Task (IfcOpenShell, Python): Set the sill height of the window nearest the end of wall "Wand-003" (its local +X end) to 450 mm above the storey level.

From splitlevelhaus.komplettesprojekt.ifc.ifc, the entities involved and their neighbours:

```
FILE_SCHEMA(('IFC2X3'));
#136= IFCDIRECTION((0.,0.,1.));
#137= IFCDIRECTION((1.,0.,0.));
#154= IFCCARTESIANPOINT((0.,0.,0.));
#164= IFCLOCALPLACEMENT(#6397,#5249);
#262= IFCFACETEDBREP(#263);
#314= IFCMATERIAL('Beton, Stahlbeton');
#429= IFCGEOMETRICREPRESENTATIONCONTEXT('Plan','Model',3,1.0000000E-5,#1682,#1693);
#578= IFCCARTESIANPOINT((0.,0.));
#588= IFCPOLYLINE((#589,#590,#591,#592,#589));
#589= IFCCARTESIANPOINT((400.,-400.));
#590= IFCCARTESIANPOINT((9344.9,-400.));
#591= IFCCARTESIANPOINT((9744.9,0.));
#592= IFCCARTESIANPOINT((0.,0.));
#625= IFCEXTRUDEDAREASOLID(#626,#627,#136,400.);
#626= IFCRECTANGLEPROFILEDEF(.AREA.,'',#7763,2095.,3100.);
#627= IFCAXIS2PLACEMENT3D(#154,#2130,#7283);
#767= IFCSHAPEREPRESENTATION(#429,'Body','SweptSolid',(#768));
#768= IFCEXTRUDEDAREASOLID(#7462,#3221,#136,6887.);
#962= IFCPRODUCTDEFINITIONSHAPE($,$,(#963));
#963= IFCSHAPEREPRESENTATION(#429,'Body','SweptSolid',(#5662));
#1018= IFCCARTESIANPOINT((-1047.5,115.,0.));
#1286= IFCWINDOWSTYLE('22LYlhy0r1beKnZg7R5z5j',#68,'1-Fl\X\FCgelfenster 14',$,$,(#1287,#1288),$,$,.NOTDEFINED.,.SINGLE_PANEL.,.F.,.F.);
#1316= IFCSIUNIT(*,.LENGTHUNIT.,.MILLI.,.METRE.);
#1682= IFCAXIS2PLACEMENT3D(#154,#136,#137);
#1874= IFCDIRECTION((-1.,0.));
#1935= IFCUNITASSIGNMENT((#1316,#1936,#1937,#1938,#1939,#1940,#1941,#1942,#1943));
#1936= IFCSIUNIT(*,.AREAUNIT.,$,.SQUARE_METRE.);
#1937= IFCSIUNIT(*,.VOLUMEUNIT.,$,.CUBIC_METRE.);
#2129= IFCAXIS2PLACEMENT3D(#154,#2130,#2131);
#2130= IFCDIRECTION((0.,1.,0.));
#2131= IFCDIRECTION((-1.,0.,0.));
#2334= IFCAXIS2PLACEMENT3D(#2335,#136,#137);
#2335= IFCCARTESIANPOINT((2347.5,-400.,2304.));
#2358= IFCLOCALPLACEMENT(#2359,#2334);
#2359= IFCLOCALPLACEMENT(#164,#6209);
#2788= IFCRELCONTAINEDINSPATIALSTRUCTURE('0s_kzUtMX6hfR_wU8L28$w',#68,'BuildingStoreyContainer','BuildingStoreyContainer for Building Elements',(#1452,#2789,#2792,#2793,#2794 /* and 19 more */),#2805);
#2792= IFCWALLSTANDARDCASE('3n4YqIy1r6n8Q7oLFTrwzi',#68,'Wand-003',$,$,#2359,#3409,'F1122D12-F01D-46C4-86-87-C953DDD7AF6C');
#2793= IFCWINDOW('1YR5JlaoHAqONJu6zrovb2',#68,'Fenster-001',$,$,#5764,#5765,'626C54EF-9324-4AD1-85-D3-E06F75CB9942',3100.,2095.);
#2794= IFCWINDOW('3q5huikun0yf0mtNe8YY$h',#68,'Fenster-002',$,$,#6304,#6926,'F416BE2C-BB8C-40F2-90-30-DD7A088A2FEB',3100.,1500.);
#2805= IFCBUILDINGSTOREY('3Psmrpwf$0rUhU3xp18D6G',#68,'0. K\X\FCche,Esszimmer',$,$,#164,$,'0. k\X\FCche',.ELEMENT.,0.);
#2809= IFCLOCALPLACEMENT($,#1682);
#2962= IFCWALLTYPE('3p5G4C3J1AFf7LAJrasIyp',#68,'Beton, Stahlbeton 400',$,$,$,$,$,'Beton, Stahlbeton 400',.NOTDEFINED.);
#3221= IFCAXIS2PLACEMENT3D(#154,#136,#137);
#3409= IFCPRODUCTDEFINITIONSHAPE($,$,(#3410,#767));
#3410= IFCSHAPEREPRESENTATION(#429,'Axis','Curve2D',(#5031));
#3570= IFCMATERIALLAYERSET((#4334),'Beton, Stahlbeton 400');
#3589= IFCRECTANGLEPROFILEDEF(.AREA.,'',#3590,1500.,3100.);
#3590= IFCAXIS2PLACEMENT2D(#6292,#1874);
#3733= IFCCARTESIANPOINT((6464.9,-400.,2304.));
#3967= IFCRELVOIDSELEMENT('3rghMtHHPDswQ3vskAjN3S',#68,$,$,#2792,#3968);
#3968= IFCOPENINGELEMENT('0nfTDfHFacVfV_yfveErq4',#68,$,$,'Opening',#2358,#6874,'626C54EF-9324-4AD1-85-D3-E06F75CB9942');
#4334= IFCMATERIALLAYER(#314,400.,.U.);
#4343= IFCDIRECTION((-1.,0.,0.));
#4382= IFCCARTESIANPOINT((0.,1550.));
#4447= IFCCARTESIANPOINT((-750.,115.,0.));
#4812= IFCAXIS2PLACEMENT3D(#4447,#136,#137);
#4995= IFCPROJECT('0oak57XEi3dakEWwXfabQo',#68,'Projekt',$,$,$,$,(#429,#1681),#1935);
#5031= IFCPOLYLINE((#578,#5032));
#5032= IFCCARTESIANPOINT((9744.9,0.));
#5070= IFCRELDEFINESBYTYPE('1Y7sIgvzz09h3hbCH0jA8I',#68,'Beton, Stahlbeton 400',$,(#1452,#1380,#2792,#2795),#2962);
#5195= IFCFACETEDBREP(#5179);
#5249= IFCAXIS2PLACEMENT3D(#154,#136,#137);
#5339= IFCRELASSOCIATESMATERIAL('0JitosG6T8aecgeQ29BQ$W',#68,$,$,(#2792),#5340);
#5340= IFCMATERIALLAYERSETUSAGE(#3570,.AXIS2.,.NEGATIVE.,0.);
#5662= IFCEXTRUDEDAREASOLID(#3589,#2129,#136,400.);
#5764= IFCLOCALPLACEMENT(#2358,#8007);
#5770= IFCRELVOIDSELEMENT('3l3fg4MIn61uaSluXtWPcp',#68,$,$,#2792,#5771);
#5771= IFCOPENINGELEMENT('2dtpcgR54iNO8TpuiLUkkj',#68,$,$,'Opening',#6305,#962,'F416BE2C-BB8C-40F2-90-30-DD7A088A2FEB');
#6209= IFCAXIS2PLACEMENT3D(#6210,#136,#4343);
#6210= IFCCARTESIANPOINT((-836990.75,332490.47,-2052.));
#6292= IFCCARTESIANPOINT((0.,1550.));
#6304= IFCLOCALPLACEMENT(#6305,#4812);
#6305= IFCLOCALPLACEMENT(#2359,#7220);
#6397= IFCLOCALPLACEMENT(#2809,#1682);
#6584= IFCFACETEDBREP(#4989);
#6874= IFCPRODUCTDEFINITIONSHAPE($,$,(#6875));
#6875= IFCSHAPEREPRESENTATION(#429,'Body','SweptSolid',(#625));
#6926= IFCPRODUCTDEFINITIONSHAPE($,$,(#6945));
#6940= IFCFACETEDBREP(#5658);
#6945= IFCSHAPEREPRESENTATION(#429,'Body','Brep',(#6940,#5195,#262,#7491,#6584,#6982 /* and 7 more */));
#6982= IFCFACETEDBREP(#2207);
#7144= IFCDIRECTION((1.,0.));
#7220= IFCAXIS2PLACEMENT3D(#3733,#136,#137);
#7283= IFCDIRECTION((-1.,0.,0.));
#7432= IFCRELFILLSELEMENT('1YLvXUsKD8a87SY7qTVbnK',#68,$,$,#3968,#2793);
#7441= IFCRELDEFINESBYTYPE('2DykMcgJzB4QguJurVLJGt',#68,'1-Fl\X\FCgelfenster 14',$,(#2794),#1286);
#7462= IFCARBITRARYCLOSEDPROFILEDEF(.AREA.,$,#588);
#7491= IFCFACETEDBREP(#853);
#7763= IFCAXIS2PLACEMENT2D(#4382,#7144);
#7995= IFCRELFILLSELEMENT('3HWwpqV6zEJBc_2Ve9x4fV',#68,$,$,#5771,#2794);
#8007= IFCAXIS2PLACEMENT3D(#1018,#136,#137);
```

```python
import numpy as np
import ifcopenshell
import ifcopenshell.api.geometry
import ifcopenshell.geom
import ifcopenshell.util.element
import ifcopenshell.util.placement
import ifcopenshell.util.shape
import ifcopenshell.util.unit

model = ifcopenshell.open("splitlevelhaus.komplettesprojekt.ifc.ifc")
unit_scale = ifcopenshell.util.unit.calculate_unit_scale(model)

window = model.by_id(2794)
opening = window.FillsVoids[0].RelatingOpeningElement
storey = ifcopenshell.util.element.get_container(window, ifc_class="IfcBuildingStorey")
level = ifcopenshell.util.placement.get_local_placement(storey.ObjectPlacement)[2, 3]

# The opening's origin need not be at the sill, so measure its lowest point.
shape = ifcopenshell.geom.create_shape(ifcopenshell.geom.settings(), opening)
bottom = ifcopenshell.util.shape.get_shape_bottom_elevation(shape, shape.geometry) / unit_scale
dz = level + 450.0 - bottom

shift = np.array([0.0, 0.0, dz])
# The window is placed relative to its opening, so it follows when the opening moves.
matrix = ifcopenshell.util.placement.get_local_placement(opening.ObjectPlacement)
matrix[:3, 3] += shift
ifcopenshell.api.geometry.edit_object_placement(
    model, product=opening, matrix=matrix, is_si=False, should_transform_children=True
)

print(f"moved by {dz * unit_scale:+.3f} m")

model.write("splitlevelhaus.komplettesprojekt.ifc_v2.ifc")
```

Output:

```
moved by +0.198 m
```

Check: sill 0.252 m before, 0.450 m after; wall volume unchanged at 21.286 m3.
